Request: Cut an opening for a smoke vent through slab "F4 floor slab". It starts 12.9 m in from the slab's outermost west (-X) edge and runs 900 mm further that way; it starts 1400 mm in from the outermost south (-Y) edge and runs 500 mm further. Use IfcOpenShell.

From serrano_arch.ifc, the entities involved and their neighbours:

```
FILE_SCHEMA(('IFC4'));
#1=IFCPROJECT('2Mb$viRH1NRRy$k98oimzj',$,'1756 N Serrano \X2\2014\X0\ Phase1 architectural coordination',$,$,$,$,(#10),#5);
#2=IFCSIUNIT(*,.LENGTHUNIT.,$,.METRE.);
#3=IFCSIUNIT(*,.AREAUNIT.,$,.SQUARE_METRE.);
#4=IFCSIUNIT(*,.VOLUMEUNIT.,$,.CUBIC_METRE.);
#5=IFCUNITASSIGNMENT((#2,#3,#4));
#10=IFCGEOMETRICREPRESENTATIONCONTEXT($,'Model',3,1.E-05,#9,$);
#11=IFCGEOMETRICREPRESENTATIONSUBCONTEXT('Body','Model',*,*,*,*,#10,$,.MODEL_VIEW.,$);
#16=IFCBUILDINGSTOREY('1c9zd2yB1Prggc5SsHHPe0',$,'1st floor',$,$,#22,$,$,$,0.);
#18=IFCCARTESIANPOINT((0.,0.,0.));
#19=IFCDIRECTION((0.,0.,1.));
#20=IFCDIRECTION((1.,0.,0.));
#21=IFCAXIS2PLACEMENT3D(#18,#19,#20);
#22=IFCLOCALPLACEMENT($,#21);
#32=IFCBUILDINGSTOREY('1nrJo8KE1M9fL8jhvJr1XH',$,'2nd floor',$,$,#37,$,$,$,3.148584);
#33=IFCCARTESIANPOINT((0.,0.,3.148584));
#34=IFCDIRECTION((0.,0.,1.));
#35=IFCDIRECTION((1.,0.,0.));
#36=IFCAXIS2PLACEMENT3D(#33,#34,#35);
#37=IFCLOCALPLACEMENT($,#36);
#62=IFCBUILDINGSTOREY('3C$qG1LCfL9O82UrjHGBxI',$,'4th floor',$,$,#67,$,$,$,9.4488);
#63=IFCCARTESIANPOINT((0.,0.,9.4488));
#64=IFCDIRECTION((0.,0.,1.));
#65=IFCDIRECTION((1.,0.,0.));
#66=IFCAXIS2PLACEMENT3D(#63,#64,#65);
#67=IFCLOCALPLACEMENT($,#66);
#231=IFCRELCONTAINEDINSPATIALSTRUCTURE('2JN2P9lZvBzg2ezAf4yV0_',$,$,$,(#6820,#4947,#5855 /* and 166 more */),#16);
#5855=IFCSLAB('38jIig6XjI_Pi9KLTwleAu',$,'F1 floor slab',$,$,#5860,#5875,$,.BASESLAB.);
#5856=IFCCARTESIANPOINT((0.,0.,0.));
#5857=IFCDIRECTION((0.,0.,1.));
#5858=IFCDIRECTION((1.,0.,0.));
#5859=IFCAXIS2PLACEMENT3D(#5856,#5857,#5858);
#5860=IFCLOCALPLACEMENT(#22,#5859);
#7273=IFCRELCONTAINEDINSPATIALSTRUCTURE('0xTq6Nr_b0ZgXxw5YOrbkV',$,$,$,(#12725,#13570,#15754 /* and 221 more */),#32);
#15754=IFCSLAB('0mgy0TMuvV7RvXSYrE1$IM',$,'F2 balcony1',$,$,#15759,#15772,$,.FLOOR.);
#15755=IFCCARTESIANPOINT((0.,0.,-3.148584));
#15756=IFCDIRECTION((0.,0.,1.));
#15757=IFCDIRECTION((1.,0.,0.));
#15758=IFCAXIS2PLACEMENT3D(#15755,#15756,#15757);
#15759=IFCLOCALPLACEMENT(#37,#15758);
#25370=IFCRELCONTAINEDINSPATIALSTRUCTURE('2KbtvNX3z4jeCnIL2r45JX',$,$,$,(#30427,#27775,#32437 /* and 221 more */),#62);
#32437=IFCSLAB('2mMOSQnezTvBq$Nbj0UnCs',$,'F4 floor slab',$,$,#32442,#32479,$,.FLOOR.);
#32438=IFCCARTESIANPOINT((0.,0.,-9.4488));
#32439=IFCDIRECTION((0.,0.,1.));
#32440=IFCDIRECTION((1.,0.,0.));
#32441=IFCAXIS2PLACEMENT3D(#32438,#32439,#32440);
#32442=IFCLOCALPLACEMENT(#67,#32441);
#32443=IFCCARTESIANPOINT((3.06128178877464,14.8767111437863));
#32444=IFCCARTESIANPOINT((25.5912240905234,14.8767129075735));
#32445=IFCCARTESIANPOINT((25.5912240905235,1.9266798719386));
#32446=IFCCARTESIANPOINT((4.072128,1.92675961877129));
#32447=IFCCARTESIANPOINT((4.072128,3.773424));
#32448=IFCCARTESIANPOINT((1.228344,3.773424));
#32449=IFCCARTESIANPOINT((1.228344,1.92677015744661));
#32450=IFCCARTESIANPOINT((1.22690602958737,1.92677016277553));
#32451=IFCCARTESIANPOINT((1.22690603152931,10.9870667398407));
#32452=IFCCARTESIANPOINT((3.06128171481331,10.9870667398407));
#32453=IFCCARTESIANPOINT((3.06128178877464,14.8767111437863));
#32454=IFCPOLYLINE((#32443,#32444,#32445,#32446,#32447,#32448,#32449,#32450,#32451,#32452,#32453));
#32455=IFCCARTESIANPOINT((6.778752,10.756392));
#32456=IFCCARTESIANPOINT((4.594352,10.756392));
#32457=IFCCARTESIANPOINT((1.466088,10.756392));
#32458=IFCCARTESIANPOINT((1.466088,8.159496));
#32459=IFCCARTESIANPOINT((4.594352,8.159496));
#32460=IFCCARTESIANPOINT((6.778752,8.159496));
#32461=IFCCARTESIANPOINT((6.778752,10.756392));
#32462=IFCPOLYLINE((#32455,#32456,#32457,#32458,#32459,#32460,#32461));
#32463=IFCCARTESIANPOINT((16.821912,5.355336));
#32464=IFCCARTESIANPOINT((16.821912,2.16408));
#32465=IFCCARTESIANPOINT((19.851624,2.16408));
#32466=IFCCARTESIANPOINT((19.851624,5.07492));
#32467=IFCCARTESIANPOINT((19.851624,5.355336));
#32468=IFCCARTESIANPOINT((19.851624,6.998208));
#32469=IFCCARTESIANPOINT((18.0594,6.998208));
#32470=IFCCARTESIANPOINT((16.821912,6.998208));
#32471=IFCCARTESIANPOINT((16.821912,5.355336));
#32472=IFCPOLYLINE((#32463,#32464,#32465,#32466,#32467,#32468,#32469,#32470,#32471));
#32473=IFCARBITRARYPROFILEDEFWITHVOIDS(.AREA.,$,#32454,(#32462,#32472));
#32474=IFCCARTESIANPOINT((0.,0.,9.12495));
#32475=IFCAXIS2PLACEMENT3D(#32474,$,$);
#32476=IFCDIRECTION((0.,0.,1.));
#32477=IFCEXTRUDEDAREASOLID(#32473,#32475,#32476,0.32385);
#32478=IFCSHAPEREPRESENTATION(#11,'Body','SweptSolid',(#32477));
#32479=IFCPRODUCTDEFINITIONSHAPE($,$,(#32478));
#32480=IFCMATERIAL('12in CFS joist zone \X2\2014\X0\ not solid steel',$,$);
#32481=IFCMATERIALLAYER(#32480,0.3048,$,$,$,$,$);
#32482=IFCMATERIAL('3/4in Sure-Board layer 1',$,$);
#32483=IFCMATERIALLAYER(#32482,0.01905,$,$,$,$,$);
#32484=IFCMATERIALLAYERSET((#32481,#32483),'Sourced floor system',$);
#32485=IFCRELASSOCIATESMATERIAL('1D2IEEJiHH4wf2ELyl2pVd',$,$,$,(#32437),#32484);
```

```python
import numpy as np
import ifcopenshell
import ifcopenshell.api.feature
import ifcopenshell.api.geometry
import ifcopenshell.api.root
import ifcopenshell.geom
import ifcopenshell.util.placement
import ifcopenshell.util.representation
import ifcopenshell.util.shape
import ifcopenshell.util.unit

model = ifcopenshell.open("serrano_arch.ifc")
unit_scale = ifcopenshell.util.unit.calculate_unit_scale(model)
settings = ifcopenshell.geom.settings()


def volume(element):
    """Net volume in cubic metres, openings subtracted."""
    shape = ifcopenshell.geom.create_shape(settings, element)
    return ifcopenshell.util.shape.get_volume(shape.geometry)


slab = model.by_guid("2mMOSQnezTvBq$Nbj0UnCs")
before = volume(slab)

# Extent in the slab's own axes, in metres. The edges named are its -X and -Y sides.
slab_shape = ifcopenshell.geom.create_shape(settings, slab)
vertices = ifcopenshell.util.shape.get_vertices(slab_shape.geometry)
x_min, y_min, bottom = vertices.min(axis=0)
top = vertices[:, 2].max()

opening = ifcopenshell.api.root.create_entity(model, ifc_class="IfcOpeningElement", name="Smoke vent opening", predefined_type="OPENING")
context = ifcopenshell.util.representation.get_context(model, "Model", "Body", "MODEL_VIEW")
width, depth = 0.9, 0.5
outline = [(0.0, 0.0), (width, 0.0), (width, depth), (0.0, depth), (0.0, 0.0)]
# Overshoot both faces by 50 mm so the cut is clean.
shape = ifcopenshell.api.geometry.add_slab_representation(
    model, context=context, depth=top - bottom + 0.1, polyline=outline
)
ifcopenshell.api.geometry.assign_representation(model, product=opening, representation=shape)

matrix = ifcopenshell.util.placement.get_local_placement(slab.ObjectPlacement)
matrix[:, 3] = matrix @ np.append(np.array([x_min + 12.9, y_min + 1.4, bottom - 0.05]) / unit_scale, 1.0)
ifcopenshell.api.geometry.edit_object_placement(model, product=opening, matrix=matrix, is_si=False)
ifcopenshell.api.feature.add_feature(model, feature=opening, element=slab)

after = volume(slab)

print(f"slab volume {before:.3f} -> {after:.3f} m3")

model.write("serrano_arch_edited.ifc")
```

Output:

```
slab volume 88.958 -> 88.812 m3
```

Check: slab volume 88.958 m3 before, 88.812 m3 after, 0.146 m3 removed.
